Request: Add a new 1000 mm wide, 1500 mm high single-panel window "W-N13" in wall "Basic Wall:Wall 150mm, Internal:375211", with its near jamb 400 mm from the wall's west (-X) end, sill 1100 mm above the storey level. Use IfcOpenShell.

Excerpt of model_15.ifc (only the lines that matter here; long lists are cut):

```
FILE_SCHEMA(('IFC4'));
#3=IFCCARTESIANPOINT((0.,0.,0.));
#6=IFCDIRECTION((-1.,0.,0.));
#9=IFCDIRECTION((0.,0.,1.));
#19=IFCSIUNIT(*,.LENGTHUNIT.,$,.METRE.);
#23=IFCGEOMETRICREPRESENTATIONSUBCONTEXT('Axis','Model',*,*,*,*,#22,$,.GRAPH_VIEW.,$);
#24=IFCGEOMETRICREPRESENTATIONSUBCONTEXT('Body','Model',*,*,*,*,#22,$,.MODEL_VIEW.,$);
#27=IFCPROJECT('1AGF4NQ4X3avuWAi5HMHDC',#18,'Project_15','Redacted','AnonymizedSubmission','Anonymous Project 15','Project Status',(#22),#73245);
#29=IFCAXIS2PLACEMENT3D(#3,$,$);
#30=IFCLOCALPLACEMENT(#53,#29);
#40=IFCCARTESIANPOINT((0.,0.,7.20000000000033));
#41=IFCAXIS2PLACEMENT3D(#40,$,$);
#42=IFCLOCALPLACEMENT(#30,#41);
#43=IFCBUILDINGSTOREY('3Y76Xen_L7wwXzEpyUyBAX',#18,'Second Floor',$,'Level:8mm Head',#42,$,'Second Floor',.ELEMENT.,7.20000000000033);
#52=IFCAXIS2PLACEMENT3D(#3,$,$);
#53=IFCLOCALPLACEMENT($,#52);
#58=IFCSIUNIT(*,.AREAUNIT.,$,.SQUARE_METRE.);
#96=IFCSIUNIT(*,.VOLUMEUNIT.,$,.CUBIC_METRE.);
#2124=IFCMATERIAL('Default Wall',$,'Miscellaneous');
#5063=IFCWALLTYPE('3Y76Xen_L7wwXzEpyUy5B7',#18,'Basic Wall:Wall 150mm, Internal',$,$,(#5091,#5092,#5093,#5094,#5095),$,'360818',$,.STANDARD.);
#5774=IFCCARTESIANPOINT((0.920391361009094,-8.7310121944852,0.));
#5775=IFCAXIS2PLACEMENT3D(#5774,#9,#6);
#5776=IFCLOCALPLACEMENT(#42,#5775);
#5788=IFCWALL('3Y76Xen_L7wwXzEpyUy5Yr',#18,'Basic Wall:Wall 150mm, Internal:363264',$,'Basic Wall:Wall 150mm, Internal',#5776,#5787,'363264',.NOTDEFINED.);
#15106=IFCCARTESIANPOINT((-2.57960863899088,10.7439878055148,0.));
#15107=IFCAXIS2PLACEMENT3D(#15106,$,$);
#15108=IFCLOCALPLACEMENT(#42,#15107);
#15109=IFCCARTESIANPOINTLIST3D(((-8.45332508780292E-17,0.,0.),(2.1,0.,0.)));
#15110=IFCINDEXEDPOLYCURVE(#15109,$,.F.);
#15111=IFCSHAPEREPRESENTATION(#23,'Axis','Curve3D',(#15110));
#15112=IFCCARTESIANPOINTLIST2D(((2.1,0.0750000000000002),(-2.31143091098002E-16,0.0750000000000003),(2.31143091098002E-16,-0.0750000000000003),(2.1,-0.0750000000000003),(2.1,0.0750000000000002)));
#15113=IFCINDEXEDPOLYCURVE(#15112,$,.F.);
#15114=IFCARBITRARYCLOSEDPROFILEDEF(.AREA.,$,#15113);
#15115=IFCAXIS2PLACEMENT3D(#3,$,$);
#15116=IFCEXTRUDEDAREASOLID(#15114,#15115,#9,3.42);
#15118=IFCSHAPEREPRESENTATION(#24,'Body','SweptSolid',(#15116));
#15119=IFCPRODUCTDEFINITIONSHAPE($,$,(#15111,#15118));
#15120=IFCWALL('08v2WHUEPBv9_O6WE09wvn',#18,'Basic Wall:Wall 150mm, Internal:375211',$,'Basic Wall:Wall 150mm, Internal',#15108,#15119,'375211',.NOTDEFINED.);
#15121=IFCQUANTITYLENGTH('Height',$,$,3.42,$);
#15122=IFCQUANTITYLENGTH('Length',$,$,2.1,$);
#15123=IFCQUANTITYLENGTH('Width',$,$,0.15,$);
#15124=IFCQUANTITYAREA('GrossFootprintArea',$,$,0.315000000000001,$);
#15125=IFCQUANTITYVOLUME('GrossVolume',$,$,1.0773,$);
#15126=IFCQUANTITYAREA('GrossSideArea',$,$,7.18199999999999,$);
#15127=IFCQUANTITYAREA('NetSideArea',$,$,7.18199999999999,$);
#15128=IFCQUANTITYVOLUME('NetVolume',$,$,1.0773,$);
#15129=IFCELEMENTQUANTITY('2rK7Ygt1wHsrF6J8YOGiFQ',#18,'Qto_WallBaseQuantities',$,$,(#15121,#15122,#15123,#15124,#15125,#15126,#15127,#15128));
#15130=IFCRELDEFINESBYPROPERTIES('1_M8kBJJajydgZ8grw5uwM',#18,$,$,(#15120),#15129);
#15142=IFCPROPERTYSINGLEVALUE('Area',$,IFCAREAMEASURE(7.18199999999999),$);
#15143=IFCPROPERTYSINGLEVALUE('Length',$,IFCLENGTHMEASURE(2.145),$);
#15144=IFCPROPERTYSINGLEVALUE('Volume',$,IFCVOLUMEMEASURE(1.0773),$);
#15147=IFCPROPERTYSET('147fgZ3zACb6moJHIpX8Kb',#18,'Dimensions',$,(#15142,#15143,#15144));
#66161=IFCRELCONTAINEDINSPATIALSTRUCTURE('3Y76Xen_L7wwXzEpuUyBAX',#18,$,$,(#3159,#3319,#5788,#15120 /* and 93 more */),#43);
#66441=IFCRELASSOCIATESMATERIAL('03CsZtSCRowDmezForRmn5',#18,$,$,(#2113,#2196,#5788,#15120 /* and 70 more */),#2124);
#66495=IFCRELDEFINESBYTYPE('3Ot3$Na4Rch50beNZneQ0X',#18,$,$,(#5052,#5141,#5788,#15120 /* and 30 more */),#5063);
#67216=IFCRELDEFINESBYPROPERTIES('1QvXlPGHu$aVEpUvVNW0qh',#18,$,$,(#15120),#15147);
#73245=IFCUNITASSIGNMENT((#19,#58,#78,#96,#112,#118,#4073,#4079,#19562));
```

```python
import numpy as np
import ifcopenshell
import ifcopenshell.api.feature
import ifcopenshell.api.geometry
import ifcopenshell.api.pset
import ifcopenshell.api.root
import ifcopenshell.api.spatial
import ifcopenshell.geom
import ifcopenshell.util.element
import ifcopenshell.util.placement
import ifcopenshell.util.representation
import ifcopenshell.util.shape
import ifcopenshell.util.unit

model = ifcopenshell.open("model_15.ifc")
unit_scale = ifcopenshell.util.unit.calculate_unit_scale(model)
area_scale = ifcopenshell.util.unit.calculate_unit_scale(model, "AREAUNIT")
volume_scale = ifcopenshell.util.unit.calculate_unit_scale(model, "VOLUMEUNIT")
settings = ifcopenshell.geom.settings()


def volume(element):
    """Net volume in cubic metres, openings subtracted."""
    shape = ifcopenshell.geom.create_shape(settings, element)
    return ifcopenshell.util.shape.get_volume(shape.geometry)


wall = model.by_guid("08v2WHUEPBv9_O6WE09wvn")
storey = ifcopenshell.util.element.get_container(wall, ifc_class="IfcBuildingStorey")
context = ifcopenshell.util.representation.get_context(model, "Model", "Body", "MODEL_VIEW")
before = volume(wall)

width, height, from_end, sill = 1, 1.5, 0.4, 1.1  # metres

# The wall runs along its own X axis, and the end named is its -X end.
wall_shape = ifcopenshell.geom.create_shape(settings, wall)
x, y, z = ifcopenshell.util.shape.get_vertices(wall_shape.geometry).T
start = x.min() + from_end
face, thickness = float(y.min()), float(y.max() - y.min())
wall_matrix = ifcopenshell.util.placement.get_local_placement(wall.ObjectPlacement)
level = ifcopenshell.util.placement.get_local_placement(storey.ObjectPlacement)[2, 3]


def in_wall(x, y):
    """Placement at x, y metres in the wall's axes, at sill height."""
    matrix = wall_matrix.copy()
    matrix[:, 3] = wall_matrix @ np.array([x / unit_scale, y / unit_scale, 0.0, 1.0])
    matrix[2, 3] = level + sill / unit_scale
    return matrix


# Opening: a box that overshoots both wall faces by 50 mm.
opening = ifcopenshell.api.root.create_entity(model, ifc_class="IfcOpeningElement", predefined_type="OPENING")
box = ifcopenshell.api.geometry.add_wall_representation(
    model, context=context, length=width, height=height, thickness=thickness + 0.1
)
ifcopenshell.api.geometry.assign_representation(model, product=opening, representation=box)
ifcopenshell.api.geometry.edit_object_placement(model, product=opening, matrix=in_wall(start, face - 0.05), is_si=False)
ifcopenshell.api.feature.add_feature(model, feature=opening, element=wall)

window = ifcopenshell.api.root.create_entity(model, ifc_class="IfcWindow", name="W-N13", predefined_type="WINDOW")
window.OverallWidth, window.OverallHeight = width / unit_scale, height / unit_scale
window.PartitioningType = "SINGLE_PANEL"
body = ifcopenshell.api.geometry.add_window_representation(
    model,
    context=context,
    overall_width=window.OverallWidth,
    overall_height=window.OverallHeight,
    partition_type="SINGLE_PANEL",
)
ifcopenshell.api.geometry.assign_representation(model, product=window, representation=body)
ifcopenshell.api.spatial.assign_container(model, products=[window], relating_structure=storey)
ifcopenshell.api.feature.add_filling(model, opening=opening, element=window)

# Centre the window in the wall's thickness.
ifcopenshell.api.geometry.edit_object_placement(model, product=window, matrix=in_wall(start, face), is_si=False)
window_shape = ifcopenshell.geom.create_shape(settings, window)
depth = ifcopenshell.util.shape.get_vertices(window_shape.geometry)[:, 1]
offset = face + thickness / 2 - (depth.min() + depth.max()) / 2
ifcopenshell.api.geometry.edit_object_placement(model, product=window, matrix=in_wall(start, offset), is_si=False)

after = volume(wall)

# Update the wall's stored quantities.
qto = model.by_id(ifcopenshell.util.element.get_pset(wall, "Qto_WallBaseQuantities", should_inherit=False)["id"])
ifcopenshell.api.pset.edit_qto(model, qto=qto, properties={
    "NetSideArea": after / thickness / area_scale,
    "NetVolume": after / volume_scale,
})
pset = model.by_id(ifcopenshell.util.element.get_pset(wall, "Dimensions", should_inherit=False)["id"])
ifcopenshell.api.pset.edit_pset(model, pset=pset, properties={
    "Area": model.create_entity("IfcAreaMeasure", after / thickness / area_scale),
    "Volume": model.create_entity("IfcVolumeMeasure", after / volume_scale),
})

print(f"wall volume {before:.3f} -> {after:.3f} m3")

model.write("model_15_edited.ifc")
```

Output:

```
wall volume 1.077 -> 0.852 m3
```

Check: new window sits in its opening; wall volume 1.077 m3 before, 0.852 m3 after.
